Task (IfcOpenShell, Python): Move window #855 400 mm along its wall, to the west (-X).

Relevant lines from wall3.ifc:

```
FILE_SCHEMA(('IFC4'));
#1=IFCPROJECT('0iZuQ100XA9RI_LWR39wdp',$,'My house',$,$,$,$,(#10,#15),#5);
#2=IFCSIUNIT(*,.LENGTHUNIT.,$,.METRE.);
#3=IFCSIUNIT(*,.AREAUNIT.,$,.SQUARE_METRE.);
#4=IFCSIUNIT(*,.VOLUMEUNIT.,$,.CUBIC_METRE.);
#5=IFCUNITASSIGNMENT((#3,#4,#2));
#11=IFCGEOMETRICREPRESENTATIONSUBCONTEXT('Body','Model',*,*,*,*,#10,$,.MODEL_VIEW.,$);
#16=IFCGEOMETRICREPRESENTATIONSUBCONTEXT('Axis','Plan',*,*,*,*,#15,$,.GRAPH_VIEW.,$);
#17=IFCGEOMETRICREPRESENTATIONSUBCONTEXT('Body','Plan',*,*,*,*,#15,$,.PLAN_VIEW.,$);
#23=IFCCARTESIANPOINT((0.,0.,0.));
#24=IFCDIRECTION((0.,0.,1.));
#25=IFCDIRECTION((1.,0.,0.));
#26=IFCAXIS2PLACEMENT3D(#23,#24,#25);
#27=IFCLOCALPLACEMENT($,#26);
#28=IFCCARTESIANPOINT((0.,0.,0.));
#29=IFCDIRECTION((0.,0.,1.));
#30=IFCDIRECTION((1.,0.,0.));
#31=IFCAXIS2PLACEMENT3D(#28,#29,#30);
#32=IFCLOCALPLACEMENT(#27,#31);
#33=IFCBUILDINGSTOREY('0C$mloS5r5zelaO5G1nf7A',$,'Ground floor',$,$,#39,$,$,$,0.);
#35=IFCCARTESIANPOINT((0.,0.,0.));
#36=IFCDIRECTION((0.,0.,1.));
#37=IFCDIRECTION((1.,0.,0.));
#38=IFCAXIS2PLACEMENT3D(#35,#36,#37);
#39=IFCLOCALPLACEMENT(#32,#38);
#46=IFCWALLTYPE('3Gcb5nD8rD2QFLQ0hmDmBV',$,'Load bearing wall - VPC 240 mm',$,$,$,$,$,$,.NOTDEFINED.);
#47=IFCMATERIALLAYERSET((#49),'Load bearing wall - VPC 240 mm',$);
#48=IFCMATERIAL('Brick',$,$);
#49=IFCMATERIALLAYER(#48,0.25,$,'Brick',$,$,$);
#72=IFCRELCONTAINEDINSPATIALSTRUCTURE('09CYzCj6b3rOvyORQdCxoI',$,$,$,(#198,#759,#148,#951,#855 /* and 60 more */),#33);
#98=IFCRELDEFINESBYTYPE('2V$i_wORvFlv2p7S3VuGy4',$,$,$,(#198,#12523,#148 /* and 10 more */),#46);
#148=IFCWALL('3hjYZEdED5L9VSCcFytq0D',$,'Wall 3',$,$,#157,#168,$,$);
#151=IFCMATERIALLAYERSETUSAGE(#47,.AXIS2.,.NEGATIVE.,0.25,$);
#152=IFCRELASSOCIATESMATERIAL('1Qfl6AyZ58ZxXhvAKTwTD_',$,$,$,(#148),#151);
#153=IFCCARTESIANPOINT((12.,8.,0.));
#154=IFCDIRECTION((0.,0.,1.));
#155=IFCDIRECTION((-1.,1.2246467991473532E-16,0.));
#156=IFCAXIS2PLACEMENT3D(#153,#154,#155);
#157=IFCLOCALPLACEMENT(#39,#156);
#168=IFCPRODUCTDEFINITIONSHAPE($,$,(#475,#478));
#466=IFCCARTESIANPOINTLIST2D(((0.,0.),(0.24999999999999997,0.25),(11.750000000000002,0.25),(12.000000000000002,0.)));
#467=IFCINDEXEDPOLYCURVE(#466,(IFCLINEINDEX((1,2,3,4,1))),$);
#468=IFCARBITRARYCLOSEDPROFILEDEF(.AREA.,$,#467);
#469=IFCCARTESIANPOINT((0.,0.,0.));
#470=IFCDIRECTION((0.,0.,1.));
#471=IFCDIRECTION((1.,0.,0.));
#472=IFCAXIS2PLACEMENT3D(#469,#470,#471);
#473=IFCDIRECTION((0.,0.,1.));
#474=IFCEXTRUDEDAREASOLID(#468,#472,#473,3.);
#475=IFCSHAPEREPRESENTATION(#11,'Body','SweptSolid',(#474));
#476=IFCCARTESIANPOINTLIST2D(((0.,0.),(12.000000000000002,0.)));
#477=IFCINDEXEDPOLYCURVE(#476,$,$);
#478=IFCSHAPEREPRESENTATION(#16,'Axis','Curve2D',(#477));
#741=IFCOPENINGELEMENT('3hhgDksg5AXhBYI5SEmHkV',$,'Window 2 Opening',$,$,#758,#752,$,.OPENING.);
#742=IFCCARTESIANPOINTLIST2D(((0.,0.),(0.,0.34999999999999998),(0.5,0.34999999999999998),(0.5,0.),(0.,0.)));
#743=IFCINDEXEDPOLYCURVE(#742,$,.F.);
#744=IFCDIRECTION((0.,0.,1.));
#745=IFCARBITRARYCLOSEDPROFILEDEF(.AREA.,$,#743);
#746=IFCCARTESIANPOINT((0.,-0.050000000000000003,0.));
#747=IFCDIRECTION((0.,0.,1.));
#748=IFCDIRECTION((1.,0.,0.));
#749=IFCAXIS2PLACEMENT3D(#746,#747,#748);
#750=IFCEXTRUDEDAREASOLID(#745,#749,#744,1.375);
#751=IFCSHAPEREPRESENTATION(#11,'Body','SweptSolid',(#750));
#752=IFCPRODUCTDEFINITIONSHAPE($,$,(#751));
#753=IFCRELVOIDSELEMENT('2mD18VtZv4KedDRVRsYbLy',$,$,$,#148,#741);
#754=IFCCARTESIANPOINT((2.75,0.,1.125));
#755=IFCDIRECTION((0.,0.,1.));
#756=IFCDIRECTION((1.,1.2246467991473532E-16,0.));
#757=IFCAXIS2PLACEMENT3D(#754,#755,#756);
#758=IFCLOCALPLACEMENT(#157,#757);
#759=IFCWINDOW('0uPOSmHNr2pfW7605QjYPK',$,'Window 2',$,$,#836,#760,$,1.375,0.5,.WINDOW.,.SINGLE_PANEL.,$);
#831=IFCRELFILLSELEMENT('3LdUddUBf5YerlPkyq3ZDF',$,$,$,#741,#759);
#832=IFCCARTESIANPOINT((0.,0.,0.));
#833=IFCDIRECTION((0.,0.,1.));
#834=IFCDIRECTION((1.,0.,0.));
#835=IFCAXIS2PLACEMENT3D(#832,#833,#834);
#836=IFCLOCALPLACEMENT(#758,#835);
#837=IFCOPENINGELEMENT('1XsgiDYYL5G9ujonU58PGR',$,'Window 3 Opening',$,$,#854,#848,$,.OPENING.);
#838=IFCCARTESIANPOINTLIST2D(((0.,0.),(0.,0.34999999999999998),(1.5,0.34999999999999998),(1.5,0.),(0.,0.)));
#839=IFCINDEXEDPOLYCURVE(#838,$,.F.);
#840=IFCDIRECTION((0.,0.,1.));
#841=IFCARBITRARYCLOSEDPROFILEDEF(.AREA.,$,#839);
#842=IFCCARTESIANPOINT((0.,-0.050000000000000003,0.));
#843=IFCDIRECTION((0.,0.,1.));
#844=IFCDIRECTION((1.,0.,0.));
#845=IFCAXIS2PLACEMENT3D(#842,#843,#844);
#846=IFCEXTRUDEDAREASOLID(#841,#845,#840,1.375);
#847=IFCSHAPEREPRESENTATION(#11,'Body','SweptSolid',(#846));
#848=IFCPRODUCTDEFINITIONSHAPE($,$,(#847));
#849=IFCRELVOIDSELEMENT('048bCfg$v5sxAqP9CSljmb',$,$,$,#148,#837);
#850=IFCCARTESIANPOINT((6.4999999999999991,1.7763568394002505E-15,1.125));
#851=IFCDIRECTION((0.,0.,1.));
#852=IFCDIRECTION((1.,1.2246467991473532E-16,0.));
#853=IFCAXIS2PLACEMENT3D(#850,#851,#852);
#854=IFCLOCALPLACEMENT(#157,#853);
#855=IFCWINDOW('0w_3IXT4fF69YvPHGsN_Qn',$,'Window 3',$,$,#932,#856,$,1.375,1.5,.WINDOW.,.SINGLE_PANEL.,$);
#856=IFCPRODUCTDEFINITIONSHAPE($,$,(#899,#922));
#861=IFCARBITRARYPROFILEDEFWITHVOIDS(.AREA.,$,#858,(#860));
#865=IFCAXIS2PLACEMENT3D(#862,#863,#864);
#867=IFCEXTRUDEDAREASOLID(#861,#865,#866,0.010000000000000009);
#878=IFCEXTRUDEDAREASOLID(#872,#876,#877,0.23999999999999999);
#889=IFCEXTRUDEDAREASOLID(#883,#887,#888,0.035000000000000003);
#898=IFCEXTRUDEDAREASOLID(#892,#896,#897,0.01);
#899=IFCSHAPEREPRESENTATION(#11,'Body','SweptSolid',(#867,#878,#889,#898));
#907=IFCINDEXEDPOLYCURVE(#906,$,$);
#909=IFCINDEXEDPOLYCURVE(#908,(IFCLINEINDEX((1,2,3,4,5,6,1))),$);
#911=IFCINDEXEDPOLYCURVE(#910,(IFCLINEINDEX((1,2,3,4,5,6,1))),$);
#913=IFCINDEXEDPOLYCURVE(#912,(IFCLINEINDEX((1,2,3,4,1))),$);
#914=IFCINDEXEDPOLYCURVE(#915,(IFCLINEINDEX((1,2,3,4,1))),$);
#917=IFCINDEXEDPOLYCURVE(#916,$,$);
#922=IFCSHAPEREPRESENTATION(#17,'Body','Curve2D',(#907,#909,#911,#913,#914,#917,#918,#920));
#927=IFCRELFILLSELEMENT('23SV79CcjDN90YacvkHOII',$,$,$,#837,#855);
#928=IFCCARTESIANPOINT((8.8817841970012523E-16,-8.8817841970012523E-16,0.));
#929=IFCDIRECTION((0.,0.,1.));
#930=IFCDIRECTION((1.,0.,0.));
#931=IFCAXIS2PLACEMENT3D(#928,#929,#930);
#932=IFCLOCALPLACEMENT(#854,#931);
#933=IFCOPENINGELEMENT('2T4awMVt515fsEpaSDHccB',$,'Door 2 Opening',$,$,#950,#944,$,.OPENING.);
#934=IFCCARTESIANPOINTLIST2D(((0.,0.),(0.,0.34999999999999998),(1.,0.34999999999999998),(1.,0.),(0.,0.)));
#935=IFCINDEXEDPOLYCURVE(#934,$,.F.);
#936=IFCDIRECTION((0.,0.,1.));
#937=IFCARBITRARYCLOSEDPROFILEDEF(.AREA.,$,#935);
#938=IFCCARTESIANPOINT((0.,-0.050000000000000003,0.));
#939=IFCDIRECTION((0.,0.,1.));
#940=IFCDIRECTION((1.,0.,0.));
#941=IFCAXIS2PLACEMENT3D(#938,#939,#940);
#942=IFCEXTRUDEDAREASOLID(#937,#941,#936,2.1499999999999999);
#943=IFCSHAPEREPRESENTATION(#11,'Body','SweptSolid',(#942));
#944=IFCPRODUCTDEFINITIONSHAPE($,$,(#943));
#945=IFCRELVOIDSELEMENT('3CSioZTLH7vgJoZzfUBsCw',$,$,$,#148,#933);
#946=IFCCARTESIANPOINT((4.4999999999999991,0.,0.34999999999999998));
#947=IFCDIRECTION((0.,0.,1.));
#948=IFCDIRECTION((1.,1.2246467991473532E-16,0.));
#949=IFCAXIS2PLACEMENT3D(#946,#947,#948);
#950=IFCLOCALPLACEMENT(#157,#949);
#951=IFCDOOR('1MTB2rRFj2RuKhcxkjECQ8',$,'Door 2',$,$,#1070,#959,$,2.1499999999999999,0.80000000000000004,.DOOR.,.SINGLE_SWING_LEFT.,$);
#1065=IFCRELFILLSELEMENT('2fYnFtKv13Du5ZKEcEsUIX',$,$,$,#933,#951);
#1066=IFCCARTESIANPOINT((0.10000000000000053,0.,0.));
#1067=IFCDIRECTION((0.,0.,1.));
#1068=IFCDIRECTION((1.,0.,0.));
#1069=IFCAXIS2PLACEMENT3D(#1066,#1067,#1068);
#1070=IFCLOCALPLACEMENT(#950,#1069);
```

```python
import ifcopenshell
import ifcopenshell.api.geometry
import ifcopenshell.util.placement
import ifcopenshell.util.unit

model = ifcopenshell.open("wall3.ifc")
unit_scale = ifcopenshell.util.unit.calculate_unit_scale(model)

window = model.by_guid("0w_3IXT4fF69YvPHGsN_Qn")
opening = window.FillsVoids[0].RelatingOpeningElement
wall = opening.VoidsElements[0].RelatingBuildingElement

wall_matrix = ifcopenshell.util.placement.get_local_placement(wall.ObjectPlacement)
shift = wall_matrix[:3, 0] * 0.4 / unit_scale
before = ifcopenshell.util.placement.get_local_placement(window.ObjectPlacement)[:3, 3].copy()

# The window is placed relative to its opening, so it follows when the opening moves.
matrix = ifcopenshell.util.placement.get_local_placement(opening.ObjectPlacement)
matrix[:3, 3] += shift
ifcopenshell.api.geometry.edit_object_placement(
    model, product=opening, matrix=matrix, is_si=False, should_transform_children=True
)

after = ifcopenshell.util.placement.get_local_placement(window.ObjectPlacement)[:3, 3]
print("window moved by", (after - before).round(3) + 0.0)

model.write("wall3_v2.ifc")
```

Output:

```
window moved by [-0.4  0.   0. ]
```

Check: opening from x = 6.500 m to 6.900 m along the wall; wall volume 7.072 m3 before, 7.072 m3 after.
